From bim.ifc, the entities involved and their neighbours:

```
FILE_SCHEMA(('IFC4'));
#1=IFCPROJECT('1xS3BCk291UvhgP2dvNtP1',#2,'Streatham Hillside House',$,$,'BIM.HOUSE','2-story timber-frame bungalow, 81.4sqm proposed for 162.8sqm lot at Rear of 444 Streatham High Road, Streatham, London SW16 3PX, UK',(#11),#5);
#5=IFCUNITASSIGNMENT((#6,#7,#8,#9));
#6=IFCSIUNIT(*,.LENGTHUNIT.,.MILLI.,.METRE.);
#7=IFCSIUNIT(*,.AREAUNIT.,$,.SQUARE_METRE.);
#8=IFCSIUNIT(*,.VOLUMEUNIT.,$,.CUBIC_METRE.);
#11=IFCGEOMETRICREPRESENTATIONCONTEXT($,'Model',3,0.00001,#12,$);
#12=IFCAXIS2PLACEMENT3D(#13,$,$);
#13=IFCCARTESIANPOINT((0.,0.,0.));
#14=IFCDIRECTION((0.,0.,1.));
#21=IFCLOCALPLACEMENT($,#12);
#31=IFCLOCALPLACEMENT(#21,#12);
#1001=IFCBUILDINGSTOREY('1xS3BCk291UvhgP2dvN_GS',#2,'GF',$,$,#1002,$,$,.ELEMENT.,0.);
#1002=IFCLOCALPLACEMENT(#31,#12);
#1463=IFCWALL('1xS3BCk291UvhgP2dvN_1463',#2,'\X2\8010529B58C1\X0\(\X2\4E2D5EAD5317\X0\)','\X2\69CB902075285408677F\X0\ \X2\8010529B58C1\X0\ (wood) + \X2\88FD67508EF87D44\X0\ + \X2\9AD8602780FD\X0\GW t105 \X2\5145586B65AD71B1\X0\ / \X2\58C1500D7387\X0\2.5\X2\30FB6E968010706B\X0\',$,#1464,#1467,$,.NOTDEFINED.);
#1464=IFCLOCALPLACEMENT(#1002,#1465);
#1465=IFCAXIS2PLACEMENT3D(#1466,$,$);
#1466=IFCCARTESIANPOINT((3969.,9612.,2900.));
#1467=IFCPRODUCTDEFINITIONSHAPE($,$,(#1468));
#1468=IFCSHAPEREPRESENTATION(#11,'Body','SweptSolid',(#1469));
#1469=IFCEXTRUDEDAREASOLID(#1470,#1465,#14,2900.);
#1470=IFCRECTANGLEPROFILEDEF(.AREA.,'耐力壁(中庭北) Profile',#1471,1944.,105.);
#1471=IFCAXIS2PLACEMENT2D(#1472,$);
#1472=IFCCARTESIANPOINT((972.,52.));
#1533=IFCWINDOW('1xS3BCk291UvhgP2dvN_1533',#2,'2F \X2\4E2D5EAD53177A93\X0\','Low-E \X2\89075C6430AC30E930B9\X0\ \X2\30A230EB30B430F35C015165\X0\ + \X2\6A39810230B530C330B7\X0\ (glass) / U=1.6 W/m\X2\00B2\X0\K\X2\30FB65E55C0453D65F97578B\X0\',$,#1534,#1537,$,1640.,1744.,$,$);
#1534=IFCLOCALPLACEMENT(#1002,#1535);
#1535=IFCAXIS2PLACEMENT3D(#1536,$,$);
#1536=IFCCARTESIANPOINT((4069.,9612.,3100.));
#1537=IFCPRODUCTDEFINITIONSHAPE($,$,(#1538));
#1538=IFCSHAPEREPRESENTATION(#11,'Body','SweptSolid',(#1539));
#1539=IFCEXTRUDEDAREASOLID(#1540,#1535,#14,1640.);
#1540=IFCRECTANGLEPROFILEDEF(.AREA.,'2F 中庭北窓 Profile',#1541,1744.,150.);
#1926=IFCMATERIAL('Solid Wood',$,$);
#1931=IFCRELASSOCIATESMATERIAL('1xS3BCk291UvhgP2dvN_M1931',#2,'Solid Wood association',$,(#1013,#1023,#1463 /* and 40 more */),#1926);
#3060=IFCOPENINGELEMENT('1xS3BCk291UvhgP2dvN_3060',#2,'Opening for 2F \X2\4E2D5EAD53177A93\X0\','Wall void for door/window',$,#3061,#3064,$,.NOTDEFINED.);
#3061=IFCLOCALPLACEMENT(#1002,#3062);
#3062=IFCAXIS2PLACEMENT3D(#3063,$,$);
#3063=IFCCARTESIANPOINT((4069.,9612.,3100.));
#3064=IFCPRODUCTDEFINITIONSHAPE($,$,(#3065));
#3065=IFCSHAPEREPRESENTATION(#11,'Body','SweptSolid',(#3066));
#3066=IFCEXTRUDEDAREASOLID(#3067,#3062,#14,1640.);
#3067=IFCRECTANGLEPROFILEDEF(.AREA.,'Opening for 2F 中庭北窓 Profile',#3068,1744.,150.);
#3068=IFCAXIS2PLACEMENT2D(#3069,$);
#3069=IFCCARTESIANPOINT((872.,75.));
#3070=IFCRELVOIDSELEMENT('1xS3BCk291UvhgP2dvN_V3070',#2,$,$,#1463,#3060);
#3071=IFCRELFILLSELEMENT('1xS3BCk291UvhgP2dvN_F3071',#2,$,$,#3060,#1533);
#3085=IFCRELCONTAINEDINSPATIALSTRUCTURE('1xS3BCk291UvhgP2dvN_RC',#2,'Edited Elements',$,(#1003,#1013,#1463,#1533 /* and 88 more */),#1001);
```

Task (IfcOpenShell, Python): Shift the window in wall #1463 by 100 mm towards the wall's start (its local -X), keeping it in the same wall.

```python
import ifcopenshell
import ifcopenshell.api.geometry
import ifcopenshell.util.placement
import ifcopenshell.util.unit

model = ifcopenshell.open("bim.ifc")
unit_scale = ifcopenshell.util.unit.calculate_unit_scale(model)

window = model.by_guid("1xS3BCk291UvhgP2dvN_1533")
opening = window.FillsVoids[0].RelatingOpeningElement
wall = opening.VoidsElements[0].RelatingBuildingElement

wall_matrix = ifcopenshell.util.placement.get_local_placement(wall.ObjectPlacement)
shift = wall_matrix[:3, 0] * -0.1 / unit_scale
before = ifcopenshell.util.placement.get_local_placement(window.ObjectPlacement)[:3, 3].copy()

# The window is not placed relative to its opening, so move both.
for product in (opening, window):
    matrix = ifcopenshell.util.placement.get_local_placement(product.ObjectPlacement)
    matrix[:3, 3] += shift
    ifcopenshell.api.geometry.edit_object_placement(model, product=product, matrix=matrix, is_si=False)

after = ifcopenshell.util.placement.get_local_placement(window.ObjectPlacement)[:3, 3]
print("window moved by", (after - before).round(3) + 0.0)

model.write("bim_v2.ifc")
```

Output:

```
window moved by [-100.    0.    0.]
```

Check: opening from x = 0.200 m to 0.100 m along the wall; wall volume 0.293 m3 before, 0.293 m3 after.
